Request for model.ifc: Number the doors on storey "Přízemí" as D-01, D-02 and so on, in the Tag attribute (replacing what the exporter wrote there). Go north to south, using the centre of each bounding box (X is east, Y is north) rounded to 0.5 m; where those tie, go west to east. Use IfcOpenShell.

First a look at what the model holds.

```python
import ifcopenshell
import ifcopenshell.util.element
import ifcopenshell.util.placement

model = ifcopenshell.open("model.ifc")
print(model.schema)
storey = next(s for s in model.by_type("IfcBuildingStorey") if s.Name == "Přízemí")
doors = [e for e in ifcopenshell.util.element.get_decomposition(storey) if e.is_a("IfcDoor")]
for e in sorted(doors, key=lambda e: e.id()):
    origin = ifcopenshell.util.placement.get_local_placement(e.ObjectPlacement)[:3, 3]
    print(e.id(), e.Tag, e.Name, origin.round(2) + 0.0, sep=" | ")
```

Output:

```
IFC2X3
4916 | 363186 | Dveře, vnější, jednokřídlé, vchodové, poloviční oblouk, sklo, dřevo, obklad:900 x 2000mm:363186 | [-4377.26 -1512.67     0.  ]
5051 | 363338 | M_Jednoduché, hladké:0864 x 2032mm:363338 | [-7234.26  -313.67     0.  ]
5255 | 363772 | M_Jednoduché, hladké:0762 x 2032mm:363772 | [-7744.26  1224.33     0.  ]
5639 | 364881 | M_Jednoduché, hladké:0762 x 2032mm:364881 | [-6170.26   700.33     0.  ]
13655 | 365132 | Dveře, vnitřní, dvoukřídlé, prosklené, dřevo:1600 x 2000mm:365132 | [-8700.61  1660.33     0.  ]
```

```python
import ifcopenshell
import ifcopenshell.geom
import ifcopenshell.util.element
import ifcopenshell.util.shape

model = ifcopenshell.open("model.ifc")
settings = ifcopenshell.geom.settings()
settings.set("use-world-coords", True)


def centre(element):
    shape = ifcopenshell.geom.create_shape(settings, element)
    return ifcopenshell.util.shape.get_bbox_centroid(shape.geometry)


storey = next(s for s in model.by_type("IfcBuildingStorey") if s.Name == "Přízemí")
doors = [e for e in ifcopenshell.util.element.get_decomposition(storey) if e.is_a("IfcDoor")]

# Insertion points can sit at a corner or the storey origin, so sort by the geometry (in metres).
centres = {e: centre(e) for e in doors}
doors.sort(key=lambda e: (-round(centres[e][1] / 0.5), centres[e][0]))

for i, e in enumerate(doors, start=1):
    number = f"D-{i:02d}"
    e.Tag = number
    print(e.id(), number)

model.write("model_v2.ifc")
```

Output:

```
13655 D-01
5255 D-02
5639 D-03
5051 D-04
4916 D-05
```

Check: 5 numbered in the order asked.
